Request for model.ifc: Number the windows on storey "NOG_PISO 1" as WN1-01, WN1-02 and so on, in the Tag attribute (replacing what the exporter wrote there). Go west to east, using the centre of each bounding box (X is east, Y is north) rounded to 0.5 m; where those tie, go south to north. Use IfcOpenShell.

First a look at what the model holds.

```python
import ifcopenshell
import ifcopenshell.util.element
import ifcopenshell.util.placement

model = ifcopenshell.open("model.ifc")
print(model.schema)
storey = next(s for s in model.by_type("IfcBuildingStorey") if s.Name == "NOG_PISO 1")
windows = [e for e in ifcopenshell.util.element.get_decomposition(storey) if e.is_a("IfcWindow")]
for e in sorted(windows, key=lambda e: e.id()):
    origin = ifcopenshell.util.placement.get_local_placement(e.ObjectPlacement)[:3, 3]
    print(e.id(), e.Tag, e.Name, origin.round(2) + 0.0, sep=" | ")
```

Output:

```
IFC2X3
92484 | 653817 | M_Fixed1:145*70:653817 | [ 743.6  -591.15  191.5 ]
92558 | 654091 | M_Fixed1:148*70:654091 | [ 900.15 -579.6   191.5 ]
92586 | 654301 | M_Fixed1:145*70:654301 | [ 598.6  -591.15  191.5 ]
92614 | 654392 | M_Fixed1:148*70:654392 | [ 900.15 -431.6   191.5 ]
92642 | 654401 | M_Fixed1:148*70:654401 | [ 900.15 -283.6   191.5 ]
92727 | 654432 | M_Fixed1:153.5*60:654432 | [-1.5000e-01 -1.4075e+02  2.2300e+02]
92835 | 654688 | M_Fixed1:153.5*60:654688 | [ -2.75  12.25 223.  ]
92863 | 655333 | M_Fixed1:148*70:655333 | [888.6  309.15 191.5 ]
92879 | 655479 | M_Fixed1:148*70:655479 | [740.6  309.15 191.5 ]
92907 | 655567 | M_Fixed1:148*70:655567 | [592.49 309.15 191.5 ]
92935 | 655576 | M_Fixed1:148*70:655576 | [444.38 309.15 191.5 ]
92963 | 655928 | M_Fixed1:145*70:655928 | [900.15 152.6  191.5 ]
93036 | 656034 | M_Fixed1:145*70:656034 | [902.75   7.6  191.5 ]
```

```python
import ifcopenshell
import ifcopenshell.geom
import ifcopenshell.util.element
import ifcopenshell.util.shape

model = ifcopenshell.open("model.ifc")
settings = ifcopenshell.geom.settings()
settings.set("use-world-coords", True)


def centre(element):
    shape = ifcopenshell.geom.create_shape(settings, element)
    return ifcopenshell.util.shape.get_bbox_centroid(shape.geometry)


storey = next(s for s in model.by_type("IfcBuildingStorey") if s.Name == "NOG_PISO 1")
windows = [e for e in ifcopenshell.util.element.get_decomposition(storey) if e.is_a("IfcWindow")]

# Insertion points can sit at a corner or the storey origin, so sort by the geometry (in metres).
centres = {e: centre(e) for e in windows}
windows.sort(key=lambda e: (round(centres[e][0] / 0.5), centres[e][1]))

for i, e in enumerate(windows, start=1):
    number = f"WN1-{i:02d}"
    e.Tag = number
    print(e.id(), number)

model.write("model_rev.ifc")
```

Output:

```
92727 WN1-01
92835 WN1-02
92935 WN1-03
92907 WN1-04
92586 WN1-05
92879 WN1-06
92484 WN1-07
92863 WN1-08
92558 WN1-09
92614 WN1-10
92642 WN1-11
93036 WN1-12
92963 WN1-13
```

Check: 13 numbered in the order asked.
